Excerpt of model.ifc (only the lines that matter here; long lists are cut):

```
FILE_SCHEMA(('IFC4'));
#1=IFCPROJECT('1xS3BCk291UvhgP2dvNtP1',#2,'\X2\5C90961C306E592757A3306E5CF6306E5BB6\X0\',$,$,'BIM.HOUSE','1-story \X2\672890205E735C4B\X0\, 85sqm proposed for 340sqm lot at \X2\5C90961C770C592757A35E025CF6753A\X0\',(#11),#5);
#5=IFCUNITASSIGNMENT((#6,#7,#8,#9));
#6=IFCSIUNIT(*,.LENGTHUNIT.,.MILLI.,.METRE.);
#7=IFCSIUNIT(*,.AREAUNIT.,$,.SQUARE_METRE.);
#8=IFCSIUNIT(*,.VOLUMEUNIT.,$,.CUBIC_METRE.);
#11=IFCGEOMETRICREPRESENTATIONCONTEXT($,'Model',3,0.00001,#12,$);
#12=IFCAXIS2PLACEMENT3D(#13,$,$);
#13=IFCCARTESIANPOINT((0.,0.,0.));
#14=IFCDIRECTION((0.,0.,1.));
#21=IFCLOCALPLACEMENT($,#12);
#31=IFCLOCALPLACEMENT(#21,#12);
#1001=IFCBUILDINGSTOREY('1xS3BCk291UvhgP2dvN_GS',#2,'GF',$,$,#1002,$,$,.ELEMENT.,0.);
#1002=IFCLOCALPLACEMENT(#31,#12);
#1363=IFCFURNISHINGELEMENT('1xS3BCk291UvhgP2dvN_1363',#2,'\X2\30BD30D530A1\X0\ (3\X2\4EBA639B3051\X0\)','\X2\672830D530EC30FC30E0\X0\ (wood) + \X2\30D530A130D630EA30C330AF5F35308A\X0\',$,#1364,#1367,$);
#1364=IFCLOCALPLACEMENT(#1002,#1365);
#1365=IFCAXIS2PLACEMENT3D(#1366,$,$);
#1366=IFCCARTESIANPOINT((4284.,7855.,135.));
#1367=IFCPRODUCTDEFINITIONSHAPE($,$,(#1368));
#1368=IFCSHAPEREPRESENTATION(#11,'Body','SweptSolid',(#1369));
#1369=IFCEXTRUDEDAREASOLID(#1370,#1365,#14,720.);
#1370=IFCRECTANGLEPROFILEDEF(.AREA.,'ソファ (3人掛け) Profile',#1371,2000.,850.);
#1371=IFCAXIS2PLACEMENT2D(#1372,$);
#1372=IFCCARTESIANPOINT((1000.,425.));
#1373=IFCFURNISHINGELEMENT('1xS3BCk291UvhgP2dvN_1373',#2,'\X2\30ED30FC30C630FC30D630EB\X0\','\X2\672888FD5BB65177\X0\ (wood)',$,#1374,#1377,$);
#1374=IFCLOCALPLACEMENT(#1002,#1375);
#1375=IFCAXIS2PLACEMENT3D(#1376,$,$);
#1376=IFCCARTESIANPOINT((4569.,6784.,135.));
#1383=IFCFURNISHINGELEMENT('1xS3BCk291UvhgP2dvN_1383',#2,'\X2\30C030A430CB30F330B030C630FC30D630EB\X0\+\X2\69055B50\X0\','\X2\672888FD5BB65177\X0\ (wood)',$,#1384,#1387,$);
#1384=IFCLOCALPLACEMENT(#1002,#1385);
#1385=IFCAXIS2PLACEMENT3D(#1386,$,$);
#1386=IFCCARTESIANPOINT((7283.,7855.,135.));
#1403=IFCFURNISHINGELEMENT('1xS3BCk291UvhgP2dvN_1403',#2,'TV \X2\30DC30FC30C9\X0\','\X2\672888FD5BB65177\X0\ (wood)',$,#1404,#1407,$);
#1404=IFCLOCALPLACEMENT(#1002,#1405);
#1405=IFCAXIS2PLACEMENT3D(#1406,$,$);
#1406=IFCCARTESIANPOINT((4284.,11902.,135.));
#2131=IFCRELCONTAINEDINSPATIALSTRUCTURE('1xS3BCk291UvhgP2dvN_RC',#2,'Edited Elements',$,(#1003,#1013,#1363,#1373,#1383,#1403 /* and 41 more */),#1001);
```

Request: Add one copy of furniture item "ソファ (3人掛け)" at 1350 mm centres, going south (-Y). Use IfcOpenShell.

```python
import numpy as np
import ifcopenshell
import ifcopenshell.api.geometry
import ifcopenshell.api.root
import ifcopenshell.util.element
import ifcopenshell.util.placement

model = ifcopenshell.open("model.ifc")


def reuse_history(source, copy):
    """copy_class also copies each property set's owner history, people and application; keep the originals."""
    for rel in copy.IsDefinedBy:
        if rel.is_a("IfcRelDefinesByProperties") and (history := rel.RelatingPropertyDefinition.OwnerHistory):
            rel.RelatingPropertyDefinition.OwnerHistory = source.OwnerHistory
            ifcopenshell.util.element.remove_deep2(model, history)


source = model.by_id(1363)
base = ifcopenshell.util.placement.get_local_placement(source.ObjectPlacement)
step = np.array([0.0, -1.0, 0.0]) * 1350.0

for i in range(1, 2):
    copy = ifcopenshell.api.root.copy_class(model, product=source)
    copy.Representation = ifcopenshell.util.element.copy_deep(
        model, source.Representation, exclude=["IfcGeometricRepresentationContext", "IfcRepresentationMap"]
    )
    reuse_history(source, copy)
    matrix = base.copy()
    matrix[:3, 3] += i * step
    print("added at", matrix[:3, 3].round(3) + 0.0)
    ifcopenshell.api.geometry.edit_object_placement(model, product=copy, matrix=matrix, is_si=False)

model.write("model_edited.ifc")
```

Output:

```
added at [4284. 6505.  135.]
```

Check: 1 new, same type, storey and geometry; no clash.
